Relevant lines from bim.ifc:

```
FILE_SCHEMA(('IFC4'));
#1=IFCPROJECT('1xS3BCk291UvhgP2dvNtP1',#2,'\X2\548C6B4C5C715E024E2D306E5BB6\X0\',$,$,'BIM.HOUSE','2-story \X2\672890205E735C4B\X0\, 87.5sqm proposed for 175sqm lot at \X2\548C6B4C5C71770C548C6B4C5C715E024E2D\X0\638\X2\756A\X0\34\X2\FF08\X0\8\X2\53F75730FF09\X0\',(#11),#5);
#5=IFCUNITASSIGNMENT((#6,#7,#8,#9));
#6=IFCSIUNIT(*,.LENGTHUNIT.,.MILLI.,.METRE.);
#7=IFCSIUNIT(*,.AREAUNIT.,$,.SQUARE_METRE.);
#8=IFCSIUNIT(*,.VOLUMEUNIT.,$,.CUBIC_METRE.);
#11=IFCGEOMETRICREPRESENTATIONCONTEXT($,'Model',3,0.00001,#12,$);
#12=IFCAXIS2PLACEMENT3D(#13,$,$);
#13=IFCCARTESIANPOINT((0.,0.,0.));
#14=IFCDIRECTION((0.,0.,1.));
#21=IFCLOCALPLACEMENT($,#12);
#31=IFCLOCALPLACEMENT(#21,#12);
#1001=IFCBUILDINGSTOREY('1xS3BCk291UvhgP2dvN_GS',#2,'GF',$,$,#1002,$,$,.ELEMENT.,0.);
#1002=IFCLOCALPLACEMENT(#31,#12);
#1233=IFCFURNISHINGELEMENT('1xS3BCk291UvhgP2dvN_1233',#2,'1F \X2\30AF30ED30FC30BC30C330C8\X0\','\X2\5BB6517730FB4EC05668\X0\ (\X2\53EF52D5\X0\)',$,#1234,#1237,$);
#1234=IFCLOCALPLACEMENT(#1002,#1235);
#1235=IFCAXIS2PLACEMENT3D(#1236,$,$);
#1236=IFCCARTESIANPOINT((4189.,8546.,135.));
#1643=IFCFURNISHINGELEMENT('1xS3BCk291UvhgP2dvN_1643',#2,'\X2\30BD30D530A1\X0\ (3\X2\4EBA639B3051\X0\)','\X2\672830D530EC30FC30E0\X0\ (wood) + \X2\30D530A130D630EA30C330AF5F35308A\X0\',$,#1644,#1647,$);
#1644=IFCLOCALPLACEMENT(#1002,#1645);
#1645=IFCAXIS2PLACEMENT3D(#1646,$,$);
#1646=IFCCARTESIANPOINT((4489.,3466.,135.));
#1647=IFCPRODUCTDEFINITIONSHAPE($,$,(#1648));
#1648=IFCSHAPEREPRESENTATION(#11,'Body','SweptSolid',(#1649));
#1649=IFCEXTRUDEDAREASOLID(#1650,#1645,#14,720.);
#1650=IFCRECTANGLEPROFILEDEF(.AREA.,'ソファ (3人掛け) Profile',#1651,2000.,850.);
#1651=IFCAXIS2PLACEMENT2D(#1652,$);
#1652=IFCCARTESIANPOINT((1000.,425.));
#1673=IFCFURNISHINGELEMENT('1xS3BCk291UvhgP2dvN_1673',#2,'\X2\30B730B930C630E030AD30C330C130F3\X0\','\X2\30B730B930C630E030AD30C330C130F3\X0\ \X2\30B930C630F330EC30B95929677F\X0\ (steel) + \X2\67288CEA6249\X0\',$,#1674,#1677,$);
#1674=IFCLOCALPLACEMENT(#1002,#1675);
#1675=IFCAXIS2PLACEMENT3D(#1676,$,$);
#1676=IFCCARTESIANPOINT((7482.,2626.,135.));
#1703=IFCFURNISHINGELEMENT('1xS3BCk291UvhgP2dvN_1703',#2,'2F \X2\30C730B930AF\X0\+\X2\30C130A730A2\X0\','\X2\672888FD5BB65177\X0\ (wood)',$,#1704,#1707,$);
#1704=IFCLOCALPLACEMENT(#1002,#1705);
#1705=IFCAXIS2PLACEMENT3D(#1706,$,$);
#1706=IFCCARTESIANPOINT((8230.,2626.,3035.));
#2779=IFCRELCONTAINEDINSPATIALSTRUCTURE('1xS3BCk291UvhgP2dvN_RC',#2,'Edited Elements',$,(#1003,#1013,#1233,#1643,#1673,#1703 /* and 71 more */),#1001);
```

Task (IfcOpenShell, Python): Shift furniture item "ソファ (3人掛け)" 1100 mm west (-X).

```python
import ifcopenshell
import ifcopenshell.api.geometry
import ifcopenshell.util.placement
import ifcopenshell.util.unit

model = ifcopenshell.open("bim.ifc")
unit_scale = ifcopenshell.util.unit.calculate_unit_scale(model)

item = model.by_guid("1xS3BCk291UvhgP2dvN_1643")
matrix = ifcopenshell.util.placement.get_local_placement(item.ObjectPlacement)
matrix[0, 3] -= 1.1 / unit_scale
ifcopenshell.api.geometry.edit_object_placement(model, product=item, matrix=matrix, is_si=False)

print(ifcopenshell.util.placement.get_local_placement(item.ObjectPlacement).round(3) + 0.0)

model.write("bim_rev.ifc")
```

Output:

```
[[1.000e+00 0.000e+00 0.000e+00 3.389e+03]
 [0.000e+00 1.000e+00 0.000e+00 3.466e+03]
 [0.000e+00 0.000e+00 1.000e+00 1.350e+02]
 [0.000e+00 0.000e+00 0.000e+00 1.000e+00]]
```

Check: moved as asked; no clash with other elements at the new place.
